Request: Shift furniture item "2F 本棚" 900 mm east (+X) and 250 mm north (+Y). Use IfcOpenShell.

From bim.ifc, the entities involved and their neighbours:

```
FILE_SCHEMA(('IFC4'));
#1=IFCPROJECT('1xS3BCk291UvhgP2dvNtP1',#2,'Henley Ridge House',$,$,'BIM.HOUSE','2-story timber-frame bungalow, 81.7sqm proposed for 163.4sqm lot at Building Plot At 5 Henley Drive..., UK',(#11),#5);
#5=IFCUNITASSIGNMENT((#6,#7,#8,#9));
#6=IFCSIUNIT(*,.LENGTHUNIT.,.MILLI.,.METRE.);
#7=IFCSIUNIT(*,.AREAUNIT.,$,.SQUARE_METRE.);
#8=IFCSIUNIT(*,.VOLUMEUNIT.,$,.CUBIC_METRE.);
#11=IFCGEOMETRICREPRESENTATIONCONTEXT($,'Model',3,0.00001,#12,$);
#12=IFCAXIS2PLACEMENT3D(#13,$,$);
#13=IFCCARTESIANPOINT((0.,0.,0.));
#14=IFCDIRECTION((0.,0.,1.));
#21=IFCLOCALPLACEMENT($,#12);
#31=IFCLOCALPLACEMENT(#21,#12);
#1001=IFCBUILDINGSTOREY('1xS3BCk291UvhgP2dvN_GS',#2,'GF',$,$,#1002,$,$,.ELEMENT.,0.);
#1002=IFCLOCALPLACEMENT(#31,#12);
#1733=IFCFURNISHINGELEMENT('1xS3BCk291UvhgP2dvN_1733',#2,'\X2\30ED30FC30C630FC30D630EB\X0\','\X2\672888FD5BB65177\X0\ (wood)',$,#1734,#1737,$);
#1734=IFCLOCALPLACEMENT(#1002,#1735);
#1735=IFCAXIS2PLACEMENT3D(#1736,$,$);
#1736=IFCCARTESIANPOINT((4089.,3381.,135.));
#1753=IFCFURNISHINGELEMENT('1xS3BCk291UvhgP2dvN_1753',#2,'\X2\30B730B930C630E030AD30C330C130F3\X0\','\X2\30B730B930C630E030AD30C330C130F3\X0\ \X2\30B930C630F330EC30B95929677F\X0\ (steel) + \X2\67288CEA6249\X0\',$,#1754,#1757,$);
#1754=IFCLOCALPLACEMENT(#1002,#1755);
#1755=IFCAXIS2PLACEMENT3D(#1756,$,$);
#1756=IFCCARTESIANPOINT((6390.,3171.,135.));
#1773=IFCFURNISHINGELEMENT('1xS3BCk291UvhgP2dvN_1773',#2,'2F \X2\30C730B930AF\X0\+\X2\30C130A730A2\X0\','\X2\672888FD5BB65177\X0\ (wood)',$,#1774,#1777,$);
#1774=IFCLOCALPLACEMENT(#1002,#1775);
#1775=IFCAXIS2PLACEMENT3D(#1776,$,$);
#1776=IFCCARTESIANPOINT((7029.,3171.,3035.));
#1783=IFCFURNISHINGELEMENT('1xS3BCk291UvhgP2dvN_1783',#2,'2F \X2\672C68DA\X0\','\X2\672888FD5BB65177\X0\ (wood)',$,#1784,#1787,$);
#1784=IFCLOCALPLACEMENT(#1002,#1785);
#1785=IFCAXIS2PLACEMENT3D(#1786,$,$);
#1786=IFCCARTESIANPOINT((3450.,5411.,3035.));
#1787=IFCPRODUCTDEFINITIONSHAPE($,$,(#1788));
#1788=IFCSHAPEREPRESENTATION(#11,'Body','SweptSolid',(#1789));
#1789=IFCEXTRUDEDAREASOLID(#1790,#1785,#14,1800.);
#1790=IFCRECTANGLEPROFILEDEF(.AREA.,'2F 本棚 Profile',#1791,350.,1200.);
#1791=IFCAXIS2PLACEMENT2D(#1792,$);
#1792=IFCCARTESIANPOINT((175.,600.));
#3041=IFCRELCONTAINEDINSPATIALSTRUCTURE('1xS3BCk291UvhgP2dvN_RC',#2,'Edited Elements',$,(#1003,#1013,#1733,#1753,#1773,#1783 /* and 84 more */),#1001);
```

```python
import ifcopenshell
import ifcopenshell.api.geometry
import ifcopenshell.util.placement

model = ifcopenshell.open("bim.ifc")

item = model.by_guid("1xS3BCk291UvhgP2dvN_1783")
matrix = ifcopenshell.util.placement.get_local_placement(item.ObjectPlacement)
matrix[0, 3] += 900.0
matrix[1, 3] += 250.0
ifcopenshell.api.geometry.edit_object_placement(model, product=item, matrix=matrix, is_si=False)

print(ifcopenshell.util.placement.get_local_placement(item.ObjectPlacement).round(3) + 0.0)

model.write("bim_edited.ifc")
```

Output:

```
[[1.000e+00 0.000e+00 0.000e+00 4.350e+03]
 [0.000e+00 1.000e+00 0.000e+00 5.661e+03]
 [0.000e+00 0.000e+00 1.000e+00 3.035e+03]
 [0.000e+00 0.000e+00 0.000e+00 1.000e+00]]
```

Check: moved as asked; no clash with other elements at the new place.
